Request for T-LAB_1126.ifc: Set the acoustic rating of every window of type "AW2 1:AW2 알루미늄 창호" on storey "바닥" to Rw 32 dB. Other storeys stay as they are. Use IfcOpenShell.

First a look at what the model holds.

```python
import ifcopenshell
import ifcopenshell.util.element

model = ifcopenshell.open("T-LAB_1126.ifc")
print(model.schema)
storey = next(s for s in model.by_type("IfcBuildingStorey") if s.Name == "바닥")
windows = [e for e in ifcopenshell.util.element.get_decomposition(storey) if e.is_a("IfcWindow")]
seen = {}
for e in windows:
    element_type = ifcopenshell.util.element.get_type(e)
    key = (element_type.Name if element_type != e and element_type else None, ifcopenshell.util.element.get_pset(e, "Pset_WindowCommon", "AcousticRating"))
    seen[key] = seen.get(key, 0) + 1
for (name, value), count in sorted(seen.items(), key=str):
    print(count, "x", name, "|", value)
```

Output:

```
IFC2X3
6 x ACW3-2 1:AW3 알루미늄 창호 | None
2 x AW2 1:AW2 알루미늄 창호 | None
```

```python
import ifcopenshell
import ifcopenshell.api.pset
import ifcopenshell.util.element

model = ifcopenshell.open("T-LAB_1126.ifc")

storey = next(s for s in model.by_type("IfcBuildingStorey") if s.Name == "바닥")
windows = [e for e in ifcopenshell.util.element.get_decomposition(storey) if e.is_a("IfcWindow")]

count = 0
for e in windows:
    element_type = ifcopenshell.util.element.get_type(e)
    if element_type in (None, e) or element_type.Name != "AW2 1:AW2 알루미늄 창호":
        continue
    # add_pset returns the element's existing set when there is one.
    pset = ifcopenshell.api.pset.add_pset(model, product=e, name="Pset_WindowCommon")
    ifcopenshell.api.pset.edit_pset(model, pset=pset, properties={"AcousticRating": "Rw 32 dB"})
    count += 1

print(count, "windows updated")

model.write("T-LAB_1126_v2.ifc")
```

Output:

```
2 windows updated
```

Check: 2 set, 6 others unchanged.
